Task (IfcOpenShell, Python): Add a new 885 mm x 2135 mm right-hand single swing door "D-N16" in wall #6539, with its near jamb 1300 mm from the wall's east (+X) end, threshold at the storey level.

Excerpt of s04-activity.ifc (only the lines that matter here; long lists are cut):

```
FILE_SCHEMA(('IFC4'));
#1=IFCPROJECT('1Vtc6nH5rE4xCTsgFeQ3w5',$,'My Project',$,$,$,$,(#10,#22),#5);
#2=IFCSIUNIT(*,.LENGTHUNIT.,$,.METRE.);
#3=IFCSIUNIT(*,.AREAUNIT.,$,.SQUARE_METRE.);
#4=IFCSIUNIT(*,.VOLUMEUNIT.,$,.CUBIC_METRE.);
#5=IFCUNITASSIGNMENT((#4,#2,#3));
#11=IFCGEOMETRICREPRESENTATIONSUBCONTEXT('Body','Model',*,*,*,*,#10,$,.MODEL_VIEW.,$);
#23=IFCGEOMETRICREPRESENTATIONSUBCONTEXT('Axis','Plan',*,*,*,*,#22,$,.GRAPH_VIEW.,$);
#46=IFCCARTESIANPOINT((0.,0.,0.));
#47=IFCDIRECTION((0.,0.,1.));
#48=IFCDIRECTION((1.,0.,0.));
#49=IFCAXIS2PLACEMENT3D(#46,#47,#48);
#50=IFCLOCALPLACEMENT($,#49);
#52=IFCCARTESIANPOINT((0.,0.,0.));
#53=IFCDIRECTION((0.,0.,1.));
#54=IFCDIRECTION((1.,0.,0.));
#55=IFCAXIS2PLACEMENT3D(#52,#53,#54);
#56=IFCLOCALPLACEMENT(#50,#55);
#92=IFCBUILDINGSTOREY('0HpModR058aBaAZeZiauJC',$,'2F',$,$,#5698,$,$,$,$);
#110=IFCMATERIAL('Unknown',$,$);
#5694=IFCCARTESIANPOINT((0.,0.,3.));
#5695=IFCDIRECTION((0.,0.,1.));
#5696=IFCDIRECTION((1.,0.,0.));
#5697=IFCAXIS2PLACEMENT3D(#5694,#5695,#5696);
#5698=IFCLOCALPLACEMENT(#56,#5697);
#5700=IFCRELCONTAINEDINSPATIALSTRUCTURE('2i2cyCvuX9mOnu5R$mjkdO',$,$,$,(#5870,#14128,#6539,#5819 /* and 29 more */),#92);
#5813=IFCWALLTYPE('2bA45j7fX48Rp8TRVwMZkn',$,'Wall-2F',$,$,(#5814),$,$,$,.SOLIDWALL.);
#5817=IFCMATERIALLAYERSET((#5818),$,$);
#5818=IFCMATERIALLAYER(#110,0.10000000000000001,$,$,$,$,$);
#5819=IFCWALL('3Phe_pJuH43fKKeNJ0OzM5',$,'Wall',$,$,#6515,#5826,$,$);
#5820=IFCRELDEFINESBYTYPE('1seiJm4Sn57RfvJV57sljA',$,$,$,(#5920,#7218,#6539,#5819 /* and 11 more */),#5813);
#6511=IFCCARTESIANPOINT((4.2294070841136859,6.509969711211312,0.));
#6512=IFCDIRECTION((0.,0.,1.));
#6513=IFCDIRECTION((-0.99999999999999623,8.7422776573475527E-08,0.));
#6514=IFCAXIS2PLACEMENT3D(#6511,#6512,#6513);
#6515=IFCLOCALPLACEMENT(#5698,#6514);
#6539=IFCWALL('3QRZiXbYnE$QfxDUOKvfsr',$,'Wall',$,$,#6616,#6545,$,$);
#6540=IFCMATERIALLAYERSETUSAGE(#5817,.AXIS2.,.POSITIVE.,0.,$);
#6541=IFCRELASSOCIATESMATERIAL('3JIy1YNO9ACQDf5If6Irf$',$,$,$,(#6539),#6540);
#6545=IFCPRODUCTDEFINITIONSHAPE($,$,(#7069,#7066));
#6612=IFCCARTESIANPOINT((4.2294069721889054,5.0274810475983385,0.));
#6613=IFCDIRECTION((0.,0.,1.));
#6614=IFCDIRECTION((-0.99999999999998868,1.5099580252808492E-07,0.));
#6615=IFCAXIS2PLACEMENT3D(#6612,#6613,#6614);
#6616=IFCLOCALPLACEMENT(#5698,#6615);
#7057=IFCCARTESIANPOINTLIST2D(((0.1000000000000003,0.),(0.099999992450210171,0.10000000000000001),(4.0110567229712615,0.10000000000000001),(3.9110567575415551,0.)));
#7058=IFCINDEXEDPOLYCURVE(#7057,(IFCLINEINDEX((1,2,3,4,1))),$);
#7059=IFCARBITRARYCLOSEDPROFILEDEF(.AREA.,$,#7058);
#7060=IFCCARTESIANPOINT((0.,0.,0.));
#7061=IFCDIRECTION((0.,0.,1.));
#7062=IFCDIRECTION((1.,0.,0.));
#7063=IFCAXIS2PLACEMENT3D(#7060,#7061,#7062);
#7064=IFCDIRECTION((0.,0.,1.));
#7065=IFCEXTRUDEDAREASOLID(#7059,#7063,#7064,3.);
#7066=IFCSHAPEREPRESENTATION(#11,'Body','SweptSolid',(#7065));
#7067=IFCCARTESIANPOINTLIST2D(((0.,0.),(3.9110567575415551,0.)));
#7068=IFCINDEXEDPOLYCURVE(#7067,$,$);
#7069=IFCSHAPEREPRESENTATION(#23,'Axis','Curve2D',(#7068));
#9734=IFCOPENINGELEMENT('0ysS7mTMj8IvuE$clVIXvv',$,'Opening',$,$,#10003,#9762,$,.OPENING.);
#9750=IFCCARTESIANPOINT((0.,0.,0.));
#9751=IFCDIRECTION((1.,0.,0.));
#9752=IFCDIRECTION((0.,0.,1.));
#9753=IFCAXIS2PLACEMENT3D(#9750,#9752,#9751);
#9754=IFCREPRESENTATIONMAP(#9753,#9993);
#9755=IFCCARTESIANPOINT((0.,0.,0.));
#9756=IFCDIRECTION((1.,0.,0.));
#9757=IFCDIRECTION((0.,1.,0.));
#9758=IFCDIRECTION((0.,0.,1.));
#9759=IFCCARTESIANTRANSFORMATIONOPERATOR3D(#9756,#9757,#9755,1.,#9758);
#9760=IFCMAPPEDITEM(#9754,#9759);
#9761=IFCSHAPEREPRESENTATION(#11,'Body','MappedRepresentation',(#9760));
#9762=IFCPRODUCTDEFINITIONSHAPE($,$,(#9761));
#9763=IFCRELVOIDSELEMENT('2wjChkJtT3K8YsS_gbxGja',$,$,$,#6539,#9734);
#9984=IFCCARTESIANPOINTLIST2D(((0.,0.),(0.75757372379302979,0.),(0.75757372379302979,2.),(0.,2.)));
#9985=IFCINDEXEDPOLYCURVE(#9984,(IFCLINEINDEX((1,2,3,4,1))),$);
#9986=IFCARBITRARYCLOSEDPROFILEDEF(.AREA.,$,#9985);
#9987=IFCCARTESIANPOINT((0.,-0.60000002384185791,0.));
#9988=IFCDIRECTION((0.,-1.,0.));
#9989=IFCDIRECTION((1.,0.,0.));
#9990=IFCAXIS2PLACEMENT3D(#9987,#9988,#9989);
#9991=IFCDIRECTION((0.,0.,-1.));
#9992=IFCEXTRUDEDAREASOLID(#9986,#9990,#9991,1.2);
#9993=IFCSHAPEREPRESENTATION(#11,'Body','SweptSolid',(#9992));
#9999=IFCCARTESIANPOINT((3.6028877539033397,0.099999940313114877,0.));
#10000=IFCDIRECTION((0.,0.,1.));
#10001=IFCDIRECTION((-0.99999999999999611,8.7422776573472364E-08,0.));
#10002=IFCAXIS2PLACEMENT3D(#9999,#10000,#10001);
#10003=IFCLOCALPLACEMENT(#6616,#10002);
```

```python
import numpy as np
import ifcopenshell
import ifcopenshell.api.feature
import ifcopenshell.api.geometry
import ifcopenshell.api.root
import ifcopenshell.api.spatial
import ifcopenshell.geom
import ifcopenshell.util.element
import ifcopenshell.util.placement
import ifcopenshell.util.representation
import ifcopenshell.util.shape
import ifcopenshell.util.unit

model = ifcopenshell.open("s04-activity.ifc")
unit_scale = ifcopenshell.util.unit.calculate_unit_scale(model)
settings = ifcopenshell.geom.settings()


def volume(element):
    """Net volume in cubic metres, openings subtracted."""
    shape = ifcopenshell.geom.create_shape(settings, element)
    return ifcopenshell.util.shape.get_volume(shape.geometry)


wall = model.by_id(6539)
storey = ifcopenshell.util.element.get_container(wall, ifc_class="IfcBuildingStorey")
context = ifcopenshell.util.representation.get_context(model, "Model", "Body", "MODEL_VIEW")
before = volume(wall)

width, height, from_end, sill = 0.885, 2.135, 1.3, 0.0  # metres

# The wall runs along its own X axis, and the end named is its -X end.
wall_shape = ifcopenshell.geom.create_shape(settings, wall)
x, y, z = ifcopenshell.util.shape.get_vertices(wall_shape.geometry).T
start = x.min() + from_end
face, thickness = float(y.min()), float(y.max() - y.min())
wall_matrix = ifcopenshell.util.placement.get_local_placement(wall.ObjectPlacement)
level = ifcopenshell.util.placement.get_local_placement(storey.ObjectPlacement)[2, 3]


def in_wall(x, y):
    """Placement at x, y metres in the wall's axes, at sill height."""
    matrix = wall_matrix.copy()
    matrix[:, 3] = wall_matrix @ np.array([x / unit_scale, y / unit_scale, 0.0, 1.0])
    matrix[2, 3] = level + sill / unit_scale
    return matrix


# Opening: a box that overshoots both wall faces by 50 mm.
opening = ifcopenshell.api.root.create_entity(model, ifc_class="IfcOpeningElement", predefined_type="OPENING")
box = ifcopenshell.api.geometry.add_wall_representation(
    model, context=context, length=width, height=height, thickness=thickness + 0.1
)
ifcopenshell.api.geometry.assign_representation(model, product=opening, representation=box)
ifcopenshell.api.geometry.edit_object_placement(model, product=opening, matrix=in_wall(start, face - 0.05), is_si=False)
ifcopenshell.api.feature.add_feature(model, feature=opening, element=wall)

door = ifcopenshell.api.root.create_entity(model, ifc_class="IfcDoor", name="D-N16", predefined_type="DOOR")
door.OverallWidth, door.OverallHeight = width / unit_scale, height / unit_scale
door.OperationType = "SINGLE_SWING_RIGHT"
body = ifcopenshell.api.geometry.add_door_representation(
    model,
    context=context,
    overall_width=door.OverallWidth,
    overall_height=door.OverallHeight,
    operation_type="SINGLE_SWING_RIGHT",
    lining_properties={"LiningDepth": thickness / unit_scale, "ThresholdDepth": thickness / unit_scale},
)
ifcopenshell.api.geometry.assign_representation(model, product=door, representation=body)
ifcopenshell.api.spatial.assign_container(model, products=[door], relating_structure=storey)
ifcopenshell.api.feature.add_filling(model, opening=opening, element=door)

# The lining spans the wall, so the door starts at the wall face.
ifcopenshell.api.geometry.edit_object_placement(model, product=door, matrix=in_wall(start, face), is_si=False)

after = volume(wall)

print(f"wall volume {before:.3f} -> {after:.3f} m3")

model.write("s04-activity_updated.ifc")
```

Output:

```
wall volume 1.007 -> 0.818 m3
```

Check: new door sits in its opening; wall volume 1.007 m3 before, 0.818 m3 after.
